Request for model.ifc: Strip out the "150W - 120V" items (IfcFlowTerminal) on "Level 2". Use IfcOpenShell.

First a look at what the model holds.

```python
import ifcopenshell
import ifcopenshell.util.element

model = ifcopenshell.open("model.ifc")
print(model.schema)
storey = next(s for s in model.by_type("IfcBuildingStorey") if s.Name == "Level 2")
terminals = [e for e in ifcopenshell.util.element.get_decomposition(storey) if e.is_a("IfcFlowTerminal")]
seen = {}
for e in terminals:
    element_type = ifcopenshell.util.element.get_type(e)
    name = element_type.Name if element_type not in (None, e) else None
    seen[name] = seen.get(name, 0) + 1
for name, count in sorted(seen.items(), key=str):
    print(count, "x", name)
```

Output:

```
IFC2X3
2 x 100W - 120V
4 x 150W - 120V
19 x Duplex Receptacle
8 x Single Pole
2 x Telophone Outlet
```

```python
import ifcopenshell
import ifcopenshell.api.root
import ifcopenshell.util.element

model = ifcopenshell.open("model.ifc")

storey = next(s for s in model.by_type("IfcBuildingStorey") if s.Name == "Level 2")
terminals = [e for e in ifcopenshell.util.element.get_decomposition(storey) if e.is_a("IfcFlowTerminal")]
targets = [e for e in terminals if (t := ifcopenshell.util.element.get_type(e)) not in (None, e) and t.Name == "150W - 120V"]

for e in targets:
    ifcopenshell.api.root.remove_product(model, product=e)
print(len(targets), "removed")

model.write("model_rev.ifc")
```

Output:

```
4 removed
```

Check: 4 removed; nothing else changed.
